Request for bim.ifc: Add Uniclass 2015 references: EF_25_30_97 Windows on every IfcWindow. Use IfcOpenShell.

First a look at what the model holds.

```python
import ifcopenshell

model = ifcopenshell.open("bim.ifc")
print(model.schema)
print("classifications:", [c.Name for c in model.by_type("IfcClassification")])
for ifc_class in ("IfcDoor", "IfcRoof", "IfcStair", "IfcWall", "IfcWindow"):
    print(ifc_class, len(model.by_type(ifc_class)))
```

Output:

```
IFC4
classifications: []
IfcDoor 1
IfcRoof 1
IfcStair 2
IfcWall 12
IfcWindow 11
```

```python
import ifcopenshell
import ifcopenshell.api.classification

model = ifcopenshell.open("bim.ifc")

system = ifcopenshell.api.classification.add_classification(model, classification="Uniclass 2015")

codes = {
    "IfcWindow": ("EF_25_30_97", "Windows"),
}
for ifc_class, (code, name) in codes.items():
    products = model.by_type(ifc_class)
    ifcopenshell.api.classification.add_reference(
        model, products=products, classification=system, identification=code, name=name
    )
    print(code, len(products))

model.write("bim_edited.ifc")
```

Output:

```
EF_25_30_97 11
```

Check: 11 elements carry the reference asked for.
